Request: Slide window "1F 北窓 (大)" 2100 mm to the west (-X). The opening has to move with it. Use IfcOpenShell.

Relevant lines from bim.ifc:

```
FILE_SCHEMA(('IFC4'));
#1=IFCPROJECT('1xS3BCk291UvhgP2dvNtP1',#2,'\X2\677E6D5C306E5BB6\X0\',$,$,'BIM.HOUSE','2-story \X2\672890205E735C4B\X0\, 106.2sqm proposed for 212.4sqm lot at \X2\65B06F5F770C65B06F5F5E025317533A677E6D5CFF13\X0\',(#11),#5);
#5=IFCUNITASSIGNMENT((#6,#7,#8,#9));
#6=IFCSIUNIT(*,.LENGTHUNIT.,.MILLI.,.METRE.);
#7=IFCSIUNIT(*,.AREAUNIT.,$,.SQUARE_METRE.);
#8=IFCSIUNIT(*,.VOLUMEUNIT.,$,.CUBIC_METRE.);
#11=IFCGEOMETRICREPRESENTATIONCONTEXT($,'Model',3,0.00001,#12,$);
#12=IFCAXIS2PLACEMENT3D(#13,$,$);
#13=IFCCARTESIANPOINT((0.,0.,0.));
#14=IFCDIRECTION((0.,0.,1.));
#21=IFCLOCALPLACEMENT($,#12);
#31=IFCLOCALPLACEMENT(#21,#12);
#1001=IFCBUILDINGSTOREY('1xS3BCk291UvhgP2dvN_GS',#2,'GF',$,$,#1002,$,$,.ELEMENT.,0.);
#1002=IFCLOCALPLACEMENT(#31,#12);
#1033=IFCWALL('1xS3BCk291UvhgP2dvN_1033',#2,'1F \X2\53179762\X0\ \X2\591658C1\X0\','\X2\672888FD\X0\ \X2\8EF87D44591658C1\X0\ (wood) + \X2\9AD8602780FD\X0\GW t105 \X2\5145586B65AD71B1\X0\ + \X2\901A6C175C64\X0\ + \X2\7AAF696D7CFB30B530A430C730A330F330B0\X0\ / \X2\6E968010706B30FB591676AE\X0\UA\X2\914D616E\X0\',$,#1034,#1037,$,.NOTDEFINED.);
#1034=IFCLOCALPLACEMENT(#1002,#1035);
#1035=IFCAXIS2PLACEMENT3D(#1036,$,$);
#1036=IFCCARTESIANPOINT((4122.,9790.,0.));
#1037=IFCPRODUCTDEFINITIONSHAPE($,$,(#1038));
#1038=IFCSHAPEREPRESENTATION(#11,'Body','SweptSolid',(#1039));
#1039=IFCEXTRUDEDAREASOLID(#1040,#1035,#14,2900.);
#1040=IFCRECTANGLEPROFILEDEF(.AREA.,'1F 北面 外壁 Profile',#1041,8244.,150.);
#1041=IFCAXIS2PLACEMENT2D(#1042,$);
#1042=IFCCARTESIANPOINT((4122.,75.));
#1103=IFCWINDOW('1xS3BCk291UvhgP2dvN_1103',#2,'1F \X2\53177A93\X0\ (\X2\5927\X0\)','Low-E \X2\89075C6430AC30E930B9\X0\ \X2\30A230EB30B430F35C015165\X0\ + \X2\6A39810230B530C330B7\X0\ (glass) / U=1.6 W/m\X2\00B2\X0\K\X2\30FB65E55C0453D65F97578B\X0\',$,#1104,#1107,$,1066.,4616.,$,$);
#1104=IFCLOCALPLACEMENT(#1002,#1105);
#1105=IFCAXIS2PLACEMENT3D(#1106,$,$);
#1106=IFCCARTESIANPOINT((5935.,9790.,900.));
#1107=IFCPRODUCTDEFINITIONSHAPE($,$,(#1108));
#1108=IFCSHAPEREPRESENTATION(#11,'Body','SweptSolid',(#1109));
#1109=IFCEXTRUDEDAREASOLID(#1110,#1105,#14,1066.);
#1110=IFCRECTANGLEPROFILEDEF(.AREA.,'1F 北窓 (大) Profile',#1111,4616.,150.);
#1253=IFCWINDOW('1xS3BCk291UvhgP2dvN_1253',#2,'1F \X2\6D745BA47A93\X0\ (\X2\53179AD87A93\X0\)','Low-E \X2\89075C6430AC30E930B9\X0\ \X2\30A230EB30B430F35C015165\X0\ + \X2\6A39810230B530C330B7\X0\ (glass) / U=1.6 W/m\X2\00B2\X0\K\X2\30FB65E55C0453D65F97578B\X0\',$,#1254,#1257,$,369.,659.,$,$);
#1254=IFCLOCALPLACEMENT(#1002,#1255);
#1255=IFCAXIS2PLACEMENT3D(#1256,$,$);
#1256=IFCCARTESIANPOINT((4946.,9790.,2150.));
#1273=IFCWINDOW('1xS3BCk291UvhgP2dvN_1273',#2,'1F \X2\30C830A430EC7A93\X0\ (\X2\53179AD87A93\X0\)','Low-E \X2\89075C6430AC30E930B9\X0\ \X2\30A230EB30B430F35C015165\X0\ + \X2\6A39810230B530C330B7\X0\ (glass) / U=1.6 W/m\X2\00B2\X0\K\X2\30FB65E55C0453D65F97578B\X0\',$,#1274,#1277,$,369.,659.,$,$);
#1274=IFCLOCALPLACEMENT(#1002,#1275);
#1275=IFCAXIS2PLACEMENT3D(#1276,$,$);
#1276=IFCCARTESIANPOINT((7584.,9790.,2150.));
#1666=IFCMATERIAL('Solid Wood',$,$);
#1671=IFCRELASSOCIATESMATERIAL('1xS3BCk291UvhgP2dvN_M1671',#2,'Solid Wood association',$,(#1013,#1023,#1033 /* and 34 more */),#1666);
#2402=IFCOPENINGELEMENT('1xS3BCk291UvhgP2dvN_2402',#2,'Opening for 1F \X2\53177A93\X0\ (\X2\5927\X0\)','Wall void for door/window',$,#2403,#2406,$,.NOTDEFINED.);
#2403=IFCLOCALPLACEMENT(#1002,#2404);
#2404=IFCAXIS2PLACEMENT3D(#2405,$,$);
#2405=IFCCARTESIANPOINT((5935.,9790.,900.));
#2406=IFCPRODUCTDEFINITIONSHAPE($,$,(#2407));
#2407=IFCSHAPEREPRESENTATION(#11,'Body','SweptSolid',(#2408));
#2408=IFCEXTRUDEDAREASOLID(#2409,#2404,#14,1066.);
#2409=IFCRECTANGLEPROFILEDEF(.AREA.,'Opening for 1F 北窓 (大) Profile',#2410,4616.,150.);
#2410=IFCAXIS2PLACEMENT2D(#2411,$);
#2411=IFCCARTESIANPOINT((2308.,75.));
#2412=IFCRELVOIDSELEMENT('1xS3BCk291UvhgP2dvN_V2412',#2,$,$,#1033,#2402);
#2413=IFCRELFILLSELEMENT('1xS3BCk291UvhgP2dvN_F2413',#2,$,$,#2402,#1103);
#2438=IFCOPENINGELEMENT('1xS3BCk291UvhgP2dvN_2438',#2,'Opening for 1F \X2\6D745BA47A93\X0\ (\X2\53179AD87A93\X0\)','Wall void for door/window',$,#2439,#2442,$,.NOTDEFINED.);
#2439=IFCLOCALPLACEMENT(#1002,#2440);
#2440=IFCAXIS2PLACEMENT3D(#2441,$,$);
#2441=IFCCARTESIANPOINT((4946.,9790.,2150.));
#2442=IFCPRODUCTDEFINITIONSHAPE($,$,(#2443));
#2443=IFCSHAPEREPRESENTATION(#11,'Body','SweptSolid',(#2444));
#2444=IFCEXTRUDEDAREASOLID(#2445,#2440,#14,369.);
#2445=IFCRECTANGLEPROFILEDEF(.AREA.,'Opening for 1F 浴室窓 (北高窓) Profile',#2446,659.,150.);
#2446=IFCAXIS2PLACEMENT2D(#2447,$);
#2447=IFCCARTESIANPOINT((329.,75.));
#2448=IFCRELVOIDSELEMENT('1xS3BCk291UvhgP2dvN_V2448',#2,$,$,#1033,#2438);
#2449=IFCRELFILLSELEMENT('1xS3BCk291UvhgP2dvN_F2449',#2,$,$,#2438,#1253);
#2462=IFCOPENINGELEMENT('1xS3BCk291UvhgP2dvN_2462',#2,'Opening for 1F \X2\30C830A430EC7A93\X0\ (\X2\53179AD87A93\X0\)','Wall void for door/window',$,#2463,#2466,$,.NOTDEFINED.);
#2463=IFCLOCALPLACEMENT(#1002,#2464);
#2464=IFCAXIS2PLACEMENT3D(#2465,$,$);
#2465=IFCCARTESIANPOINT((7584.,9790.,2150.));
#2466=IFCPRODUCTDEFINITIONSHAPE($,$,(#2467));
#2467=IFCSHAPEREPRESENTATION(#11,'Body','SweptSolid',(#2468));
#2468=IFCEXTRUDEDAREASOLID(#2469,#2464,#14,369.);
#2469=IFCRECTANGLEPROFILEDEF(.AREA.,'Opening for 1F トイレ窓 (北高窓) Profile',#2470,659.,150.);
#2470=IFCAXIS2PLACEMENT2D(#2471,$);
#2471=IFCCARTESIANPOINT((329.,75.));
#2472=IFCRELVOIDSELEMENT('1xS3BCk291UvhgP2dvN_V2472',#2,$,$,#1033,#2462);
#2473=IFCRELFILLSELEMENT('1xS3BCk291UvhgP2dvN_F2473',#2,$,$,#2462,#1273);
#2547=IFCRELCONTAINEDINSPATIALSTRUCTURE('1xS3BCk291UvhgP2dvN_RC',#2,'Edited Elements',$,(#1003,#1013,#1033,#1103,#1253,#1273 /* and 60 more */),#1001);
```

```python
import ifcopenshell
import ifcopenshell.api.geometry
import ifcopenshell.util.placement
import ifcopenshell.util.unit

model = ifcopenshell.open("bim.ifc")
unit_scale = ifcopenshell.util.unit.calculate_unit_scale(model)

window = model.by_guid("1xS3BCk291UvhgP2dvN_1103")
opening = window.FillsVoids[0].RelatingOpeningElement
wall = opening.VoidsElements[0].RelatingBuildingElement

wall_matrix = ifcopenshell.util.placement.get_local_placement(wall.ObjectPlacement)
shift = wall_matrix[:3, 0] * -2.1 / unit_scale
before = ifcopenshell.util.placement.get_local_placement(window.ObjectPlacement)[:3, 3].copy()

# The window is not placed relative to its opening, so move both.
for product in (opening, window):
    matrix = ifcopenshell.util.placement.get_local_placement(product.ObjectPlacement)
    matrix[:3, 3] += shift
    ifcopenshell.api.geometry.edit_object_placement(model, product=product, matrix=matrix, is_si=False)

after = ifcopenshell.util.placement.get_local_placement(window.ObjectPlacement)[:3, 3]
print("window moved by", (after - before).round(3) + 0.0)

model.write("bim_updated.ifc")
```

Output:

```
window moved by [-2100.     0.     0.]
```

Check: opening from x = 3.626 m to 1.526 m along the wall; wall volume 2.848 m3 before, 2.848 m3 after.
